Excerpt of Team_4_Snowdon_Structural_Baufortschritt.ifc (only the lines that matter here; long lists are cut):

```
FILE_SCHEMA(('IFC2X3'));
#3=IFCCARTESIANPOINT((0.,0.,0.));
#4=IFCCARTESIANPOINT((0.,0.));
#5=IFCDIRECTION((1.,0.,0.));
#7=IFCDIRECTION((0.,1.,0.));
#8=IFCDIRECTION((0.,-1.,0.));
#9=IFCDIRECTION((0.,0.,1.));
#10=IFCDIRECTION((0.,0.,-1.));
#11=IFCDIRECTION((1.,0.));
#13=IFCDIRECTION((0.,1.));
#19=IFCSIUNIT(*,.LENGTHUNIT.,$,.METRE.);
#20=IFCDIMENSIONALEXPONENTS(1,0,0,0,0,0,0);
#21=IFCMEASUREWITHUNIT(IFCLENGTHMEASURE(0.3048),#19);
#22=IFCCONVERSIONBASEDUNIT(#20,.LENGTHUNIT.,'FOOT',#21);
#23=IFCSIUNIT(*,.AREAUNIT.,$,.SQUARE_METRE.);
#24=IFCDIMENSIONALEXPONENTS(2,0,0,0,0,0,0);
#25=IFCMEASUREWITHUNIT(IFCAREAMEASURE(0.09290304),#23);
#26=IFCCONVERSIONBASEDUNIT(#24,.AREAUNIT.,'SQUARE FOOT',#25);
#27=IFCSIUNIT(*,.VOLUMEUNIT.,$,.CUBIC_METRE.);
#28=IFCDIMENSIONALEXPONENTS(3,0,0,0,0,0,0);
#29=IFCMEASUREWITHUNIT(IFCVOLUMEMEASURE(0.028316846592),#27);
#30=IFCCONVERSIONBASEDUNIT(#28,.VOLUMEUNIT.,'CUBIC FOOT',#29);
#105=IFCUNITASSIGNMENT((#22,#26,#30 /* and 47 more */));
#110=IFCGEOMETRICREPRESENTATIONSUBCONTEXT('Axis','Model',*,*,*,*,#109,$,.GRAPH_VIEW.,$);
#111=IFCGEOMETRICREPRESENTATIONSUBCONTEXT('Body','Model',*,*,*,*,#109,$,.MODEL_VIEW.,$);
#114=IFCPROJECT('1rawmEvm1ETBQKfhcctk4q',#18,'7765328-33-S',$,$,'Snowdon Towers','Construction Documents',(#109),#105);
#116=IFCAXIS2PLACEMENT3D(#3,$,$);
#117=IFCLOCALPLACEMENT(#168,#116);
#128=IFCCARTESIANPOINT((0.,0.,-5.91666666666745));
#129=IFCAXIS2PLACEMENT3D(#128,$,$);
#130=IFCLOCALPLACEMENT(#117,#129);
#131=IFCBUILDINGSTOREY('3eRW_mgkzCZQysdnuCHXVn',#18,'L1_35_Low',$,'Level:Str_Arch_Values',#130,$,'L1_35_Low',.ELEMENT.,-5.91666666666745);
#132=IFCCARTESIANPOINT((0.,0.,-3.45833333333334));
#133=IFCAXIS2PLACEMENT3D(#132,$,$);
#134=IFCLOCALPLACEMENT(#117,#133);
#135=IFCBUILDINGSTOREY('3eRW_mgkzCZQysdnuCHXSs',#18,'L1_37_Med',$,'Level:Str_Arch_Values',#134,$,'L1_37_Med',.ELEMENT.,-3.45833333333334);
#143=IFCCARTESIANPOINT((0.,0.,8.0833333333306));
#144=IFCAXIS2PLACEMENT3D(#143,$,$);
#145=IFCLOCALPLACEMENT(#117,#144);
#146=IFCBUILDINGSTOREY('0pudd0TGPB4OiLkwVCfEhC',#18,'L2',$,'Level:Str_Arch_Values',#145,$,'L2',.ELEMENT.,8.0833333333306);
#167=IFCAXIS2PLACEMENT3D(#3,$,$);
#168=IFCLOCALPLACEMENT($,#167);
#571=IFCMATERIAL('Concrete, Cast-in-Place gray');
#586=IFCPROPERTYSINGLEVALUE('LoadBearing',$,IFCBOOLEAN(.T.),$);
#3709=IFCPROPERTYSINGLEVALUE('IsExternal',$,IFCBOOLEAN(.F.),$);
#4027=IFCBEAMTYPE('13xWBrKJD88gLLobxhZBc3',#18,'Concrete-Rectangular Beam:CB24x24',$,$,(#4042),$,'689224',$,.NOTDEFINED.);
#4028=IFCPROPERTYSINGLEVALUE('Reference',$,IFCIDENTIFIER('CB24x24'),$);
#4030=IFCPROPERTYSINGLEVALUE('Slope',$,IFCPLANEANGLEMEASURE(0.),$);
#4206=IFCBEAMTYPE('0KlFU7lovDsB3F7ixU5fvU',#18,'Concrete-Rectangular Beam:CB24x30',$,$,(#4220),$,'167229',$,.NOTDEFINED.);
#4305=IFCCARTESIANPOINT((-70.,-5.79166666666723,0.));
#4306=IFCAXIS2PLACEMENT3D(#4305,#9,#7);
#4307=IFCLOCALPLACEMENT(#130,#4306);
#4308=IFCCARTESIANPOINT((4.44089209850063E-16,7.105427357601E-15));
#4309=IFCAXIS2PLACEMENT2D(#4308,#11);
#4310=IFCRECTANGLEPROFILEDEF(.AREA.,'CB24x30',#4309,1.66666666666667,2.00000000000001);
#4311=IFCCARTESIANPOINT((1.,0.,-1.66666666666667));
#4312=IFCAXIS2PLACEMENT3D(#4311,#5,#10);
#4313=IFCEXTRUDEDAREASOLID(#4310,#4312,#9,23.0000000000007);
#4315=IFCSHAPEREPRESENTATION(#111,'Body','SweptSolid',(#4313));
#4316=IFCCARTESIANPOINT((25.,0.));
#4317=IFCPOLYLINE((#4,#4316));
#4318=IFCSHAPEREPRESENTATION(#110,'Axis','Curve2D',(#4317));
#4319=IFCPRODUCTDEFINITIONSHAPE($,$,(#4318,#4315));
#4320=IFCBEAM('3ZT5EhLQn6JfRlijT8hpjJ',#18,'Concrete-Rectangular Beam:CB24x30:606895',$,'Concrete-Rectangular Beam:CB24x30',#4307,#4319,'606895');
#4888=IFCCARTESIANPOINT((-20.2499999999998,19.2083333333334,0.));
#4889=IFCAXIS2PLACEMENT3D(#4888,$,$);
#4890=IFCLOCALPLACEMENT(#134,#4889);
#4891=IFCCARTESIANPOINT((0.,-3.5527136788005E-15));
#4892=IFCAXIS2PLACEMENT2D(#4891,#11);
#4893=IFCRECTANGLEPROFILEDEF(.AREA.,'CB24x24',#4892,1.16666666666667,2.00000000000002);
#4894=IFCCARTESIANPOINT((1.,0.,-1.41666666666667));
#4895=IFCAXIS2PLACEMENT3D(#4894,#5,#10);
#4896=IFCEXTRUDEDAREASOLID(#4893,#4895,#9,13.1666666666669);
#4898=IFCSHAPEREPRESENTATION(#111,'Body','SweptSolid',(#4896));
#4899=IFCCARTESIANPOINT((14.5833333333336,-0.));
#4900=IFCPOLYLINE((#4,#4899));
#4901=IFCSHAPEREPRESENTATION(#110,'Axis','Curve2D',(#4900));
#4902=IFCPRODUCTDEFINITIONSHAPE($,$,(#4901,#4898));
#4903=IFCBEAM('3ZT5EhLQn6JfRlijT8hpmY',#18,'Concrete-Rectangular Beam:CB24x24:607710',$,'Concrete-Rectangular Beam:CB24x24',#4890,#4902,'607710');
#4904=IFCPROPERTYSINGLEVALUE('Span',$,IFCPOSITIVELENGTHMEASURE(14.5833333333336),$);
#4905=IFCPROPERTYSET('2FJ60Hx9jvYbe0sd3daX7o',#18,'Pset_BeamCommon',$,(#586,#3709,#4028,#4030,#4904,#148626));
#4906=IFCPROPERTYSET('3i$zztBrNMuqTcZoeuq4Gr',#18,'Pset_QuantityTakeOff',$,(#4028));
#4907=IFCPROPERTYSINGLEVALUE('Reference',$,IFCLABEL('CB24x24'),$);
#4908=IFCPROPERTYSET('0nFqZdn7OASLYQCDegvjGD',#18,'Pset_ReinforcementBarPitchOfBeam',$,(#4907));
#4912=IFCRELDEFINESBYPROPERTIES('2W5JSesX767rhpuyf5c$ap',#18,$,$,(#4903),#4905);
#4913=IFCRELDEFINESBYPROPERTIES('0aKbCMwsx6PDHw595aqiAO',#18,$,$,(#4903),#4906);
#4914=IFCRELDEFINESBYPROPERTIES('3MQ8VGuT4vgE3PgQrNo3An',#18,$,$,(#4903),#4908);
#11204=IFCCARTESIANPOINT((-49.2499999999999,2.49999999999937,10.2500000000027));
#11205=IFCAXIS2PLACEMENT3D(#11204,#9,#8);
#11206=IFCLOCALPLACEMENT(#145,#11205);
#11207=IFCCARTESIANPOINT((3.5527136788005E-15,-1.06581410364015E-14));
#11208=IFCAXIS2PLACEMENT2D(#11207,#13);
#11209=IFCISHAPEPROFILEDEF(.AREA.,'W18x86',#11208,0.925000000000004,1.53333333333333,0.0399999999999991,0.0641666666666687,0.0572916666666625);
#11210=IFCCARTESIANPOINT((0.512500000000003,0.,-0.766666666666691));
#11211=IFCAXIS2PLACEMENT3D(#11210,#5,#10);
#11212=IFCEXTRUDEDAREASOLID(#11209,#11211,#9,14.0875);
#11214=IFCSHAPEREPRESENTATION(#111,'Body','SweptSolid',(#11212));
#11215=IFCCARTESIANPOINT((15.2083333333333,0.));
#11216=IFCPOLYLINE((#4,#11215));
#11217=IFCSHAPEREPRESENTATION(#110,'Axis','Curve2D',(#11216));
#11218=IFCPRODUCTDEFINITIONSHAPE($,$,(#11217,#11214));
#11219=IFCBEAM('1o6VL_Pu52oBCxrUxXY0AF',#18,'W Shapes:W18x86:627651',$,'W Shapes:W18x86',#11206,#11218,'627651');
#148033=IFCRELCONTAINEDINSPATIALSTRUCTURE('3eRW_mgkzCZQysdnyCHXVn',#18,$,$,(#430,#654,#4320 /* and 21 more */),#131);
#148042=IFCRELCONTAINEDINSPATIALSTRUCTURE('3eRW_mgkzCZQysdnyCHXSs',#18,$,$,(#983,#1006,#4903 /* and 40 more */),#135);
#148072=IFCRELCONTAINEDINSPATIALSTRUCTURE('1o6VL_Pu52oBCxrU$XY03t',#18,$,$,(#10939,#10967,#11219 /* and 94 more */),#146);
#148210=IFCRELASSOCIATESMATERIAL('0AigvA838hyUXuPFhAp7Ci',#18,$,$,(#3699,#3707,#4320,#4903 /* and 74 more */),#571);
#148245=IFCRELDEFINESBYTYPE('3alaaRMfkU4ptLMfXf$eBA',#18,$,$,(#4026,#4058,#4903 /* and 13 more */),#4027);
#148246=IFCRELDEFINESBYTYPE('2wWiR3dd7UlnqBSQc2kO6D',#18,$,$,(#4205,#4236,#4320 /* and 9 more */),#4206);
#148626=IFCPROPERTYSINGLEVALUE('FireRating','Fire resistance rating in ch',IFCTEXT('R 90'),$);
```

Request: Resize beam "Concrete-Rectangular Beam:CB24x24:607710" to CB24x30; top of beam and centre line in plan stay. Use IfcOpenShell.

```python
import ifcopenshell
import ifcopenshell.api.pset
import ifcopenshell.api.type
import ifcopenshell.util.element
import ifcopenshell.util.representation

model = ifcopenshell.open("Team_4_Snowdon_Structural_Baufortschritt.ifc")

member = model.by_guid("3ZT5EhLQn6JfRlijT8hpmY")
source = next(p for p in model.by_type("IfcRectangleProfileDef") if p.ProfileName == "CB24x30")

body = ifcopenshell.util.representation.get_representation(member, "Model", "Body")
solid = body.Items[0]
old_profile = solid.SweptArea

# Copy the section's sizes but keep this member's own profile position.
profile = ifcopenshell.util.element.copy(model, source)
# Profiles are centred, so shift by half the change in depth to hold the top.
shift = (old_profile.XDim - profile.XDim) / 2
x, y = old_profile.Position.Location.Coordinates
up = (-1.0, 0.0)  # upwards, in the solid's own plane
location = model.createIfcCartesianPoint((x + up[0] * shift, y + up[1] * shift))
profile.Position = model.createIfcAxis2Placement2D(location, old_profile.Position.RefDirection)
solid.SweptArea = profile
if not model.get_total_inverses(old_profile):
    ifcopenshell.util.element.remove_deep2(model, old_profile)

new_type = model.by_id(4206)
ifcopenshell.api.type.assign_type(
    model, related_objects=[member], relating_type=new_type, should_map_representations=False
)
member.Name = member.Name.replace("CB24x24", "CB24x30")
member.ObjectType = "Concrete-Rectangular Beam:CB24x30"
pset = model.by_id(ifcopenshell.util.element.get_pset(member, "Pset_BeamCommon", should_inherit=False)["id"])
ifcopenshell.api.pset.edit_pset(model, pset=pset, properties={"Reference": "CB24x30"})
pset = model.by_id(ifcopenshell.util.element.get_pset(member, "Pset_QuantityTakeOff", should_inherit=False)["id"])
ifcopenshell.api.pset.edit_pset(model, pset=pset, properties={"Reference": "CB24x30"})
pset = model.by_id(ifcopenshell.util.element.get_pset(member, "Pset_ReinforcementBarPitchOfBeam", should_inherit=False)["id"])
ifcopenshell.api.pset.edit_pset(model, pset=pset, properties={"Reference": "CB24x30"})

print(solid.SweptArea)

model.write("Team_4_Snowdon_Structural_Baufortschritt_edited.ifc")
```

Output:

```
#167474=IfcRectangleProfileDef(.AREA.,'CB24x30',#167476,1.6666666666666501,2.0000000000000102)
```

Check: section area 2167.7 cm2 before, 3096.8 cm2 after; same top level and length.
